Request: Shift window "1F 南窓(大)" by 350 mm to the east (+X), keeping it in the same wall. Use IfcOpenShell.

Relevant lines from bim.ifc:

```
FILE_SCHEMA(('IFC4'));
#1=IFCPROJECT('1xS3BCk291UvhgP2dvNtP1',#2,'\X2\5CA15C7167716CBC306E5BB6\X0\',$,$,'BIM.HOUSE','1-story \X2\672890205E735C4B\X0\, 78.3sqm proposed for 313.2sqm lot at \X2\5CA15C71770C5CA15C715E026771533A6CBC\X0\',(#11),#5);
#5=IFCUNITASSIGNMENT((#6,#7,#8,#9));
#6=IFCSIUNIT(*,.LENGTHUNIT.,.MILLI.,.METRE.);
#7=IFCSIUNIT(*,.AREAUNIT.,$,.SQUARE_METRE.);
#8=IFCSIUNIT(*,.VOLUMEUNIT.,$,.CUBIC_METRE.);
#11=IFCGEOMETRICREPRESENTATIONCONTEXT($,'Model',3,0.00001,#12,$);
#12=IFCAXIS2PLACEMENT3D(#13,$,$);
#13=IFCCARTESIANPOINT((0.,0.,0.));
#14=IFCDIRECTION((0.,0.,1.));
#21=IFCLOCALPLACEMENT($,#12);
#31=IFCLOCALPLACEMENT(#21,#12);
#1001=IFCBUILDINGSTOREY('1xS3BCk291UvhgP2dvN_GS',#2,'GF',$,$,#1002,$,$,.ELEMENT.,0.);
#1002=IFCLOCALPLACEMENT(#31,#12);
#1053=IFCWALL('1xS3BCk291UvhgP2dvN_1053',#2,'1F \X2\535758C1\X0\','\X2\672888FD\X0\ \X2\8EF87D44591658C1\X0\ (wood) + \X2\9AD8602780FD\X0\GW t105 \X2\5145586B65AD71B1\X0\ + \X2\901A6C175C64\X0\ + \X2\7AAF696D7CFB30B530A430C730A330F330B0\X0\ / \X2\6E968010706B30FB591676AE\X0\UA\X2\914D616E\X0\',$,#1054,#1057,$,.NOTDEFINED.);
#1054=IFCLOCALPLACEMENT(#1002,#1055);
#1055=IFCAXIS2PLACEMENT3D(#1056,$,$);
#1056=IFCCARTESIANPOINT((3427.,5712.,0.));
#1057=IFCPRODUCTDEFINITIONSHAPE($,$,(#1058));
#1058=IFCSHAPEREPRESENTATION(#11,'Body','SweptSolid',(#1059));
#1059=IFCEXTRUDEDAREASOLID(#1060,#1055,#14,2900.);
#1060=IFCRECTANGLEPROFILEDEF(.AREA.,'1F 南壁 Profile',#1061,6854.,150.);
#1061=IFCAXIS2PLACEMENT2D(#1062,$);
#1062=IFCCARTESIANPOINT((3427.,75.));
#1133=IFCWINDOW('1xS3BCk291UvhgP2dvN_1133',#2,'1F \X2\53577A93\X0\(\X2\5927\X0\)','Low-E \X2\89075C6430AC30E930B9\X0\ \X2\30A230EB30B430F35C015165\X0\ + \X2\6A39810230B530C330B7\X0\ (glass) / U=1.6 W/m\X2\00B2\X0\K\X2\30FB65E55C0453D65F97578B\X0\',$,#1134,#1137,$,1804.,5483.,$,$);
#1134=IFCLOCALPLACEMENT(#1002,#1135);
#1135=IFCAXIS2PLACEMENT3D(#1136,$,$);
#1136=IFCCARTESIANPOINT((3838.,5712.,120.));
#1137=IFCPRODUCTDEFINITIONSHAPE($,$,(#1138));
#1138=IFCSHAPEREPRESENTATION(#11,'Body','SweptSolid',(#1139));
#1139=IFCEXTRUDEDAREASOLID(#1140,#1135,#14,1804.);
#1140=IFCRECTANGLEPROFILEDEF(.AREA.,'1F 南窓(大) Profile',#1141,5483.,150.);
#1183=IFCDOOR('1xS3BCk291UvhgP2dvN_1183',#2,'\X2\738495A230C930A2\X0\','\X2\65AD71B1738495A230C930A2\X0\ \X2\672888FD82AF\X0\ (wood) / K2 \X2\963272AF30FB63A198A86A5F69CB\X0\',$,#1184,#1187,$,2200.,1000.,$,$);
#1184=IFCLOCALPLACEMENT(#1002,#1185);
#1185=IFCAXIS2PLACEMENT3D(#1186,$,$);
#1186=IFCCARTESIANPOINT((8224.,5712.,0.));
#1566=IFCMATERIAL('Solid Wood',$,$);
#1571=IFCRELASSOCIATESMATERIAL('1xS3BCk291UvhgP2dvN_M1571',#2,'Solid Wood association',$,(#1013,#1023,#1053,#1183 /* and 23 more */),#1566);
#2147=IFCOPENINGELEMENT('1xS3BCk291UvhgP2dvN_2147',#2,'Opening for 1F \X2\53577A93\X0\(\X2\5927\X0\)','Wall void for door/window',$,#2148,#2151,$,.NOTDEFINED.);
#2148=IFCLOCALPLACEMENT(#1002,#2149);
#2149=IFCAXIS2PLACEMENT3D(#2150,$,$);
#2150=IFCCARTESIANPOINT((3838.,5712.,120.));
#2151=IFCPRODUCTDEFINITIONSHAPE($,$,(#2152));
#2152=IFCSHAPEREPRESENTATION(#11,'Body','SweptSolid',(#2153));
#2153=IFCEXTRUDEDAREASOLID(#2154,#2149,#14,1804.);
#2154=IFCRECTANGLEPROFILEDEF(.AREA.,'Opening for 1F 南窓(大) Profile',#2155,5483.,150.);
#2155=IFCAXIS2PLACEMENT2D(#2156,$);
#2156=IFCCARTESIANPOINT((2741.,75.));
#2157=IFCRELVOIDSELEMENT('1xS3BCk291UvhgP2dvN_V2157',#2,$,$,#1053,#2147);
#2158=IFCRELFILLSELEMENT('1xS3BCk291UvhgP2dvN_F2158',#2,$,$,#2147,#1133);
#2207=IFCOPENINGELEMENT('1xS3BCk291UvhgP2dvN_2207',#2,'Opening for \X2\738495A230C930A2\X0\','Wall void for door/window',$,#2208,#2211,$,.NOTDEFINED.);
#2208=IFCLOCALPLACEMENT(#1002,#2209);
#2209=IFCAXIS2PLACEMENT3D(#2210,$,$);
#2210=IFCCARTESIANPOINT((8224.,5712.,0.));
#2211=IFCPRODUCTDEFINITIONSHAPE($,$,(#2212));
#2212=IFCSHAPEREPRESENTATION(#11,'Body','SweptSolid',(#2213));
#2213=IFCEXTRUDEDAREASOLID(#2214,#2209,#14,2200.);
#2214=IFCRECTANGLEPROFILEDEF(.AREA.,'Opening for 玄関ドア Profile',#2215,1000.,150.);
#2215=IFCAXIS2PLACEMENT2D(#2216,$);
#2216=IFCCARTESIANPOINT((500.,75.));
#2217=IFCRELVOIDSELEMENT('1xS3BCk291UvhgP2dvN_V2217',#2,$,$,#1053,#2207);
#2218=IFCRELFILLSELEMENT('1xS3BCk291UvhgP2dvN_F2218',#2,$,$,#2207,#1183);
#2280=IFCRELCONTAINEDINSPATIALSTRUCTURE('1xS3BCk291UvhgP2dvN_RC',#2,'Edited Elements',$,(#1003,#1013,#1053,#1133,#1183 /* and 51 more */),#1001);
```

```python
import ifcopenshell
import ifcopenshell.api.geometry
import ifcopenshell.util.placement
import ifcopenshell.util.unit

model = ifcopenshell.open("bim.ifc")
unit_scale = ifcopenshell.util.unit.calculate_unit_scale(model)

window = model.by_guid("1xS3BCk291UvhgP2dvN_1133")
opening = window.FillsVoids[0].RelatingOpeningElement
wall = opening.VoidsElements[0].RelatingBuildingElement

wall_matrix = ifcopenshell.util.placement.get_local_placement(wall.ObjectPlacement)
shift = wall_matrix[:3, 0] * 0.35 / unit_scale
before = ifcopenshell.util.placement.get_local_placement(window.ObjectPlacement)[:3, 3].copy()

# The window is not placed relative to its opening, so move both.
for product in (opening, window):
    matrix = ifcopenshell.util.placement.get_local_placement(product.ObjectPlacement)
    matrix[:3, 3] += shift
    ifcopenshell.api.geometry.edit_object_placement(model, product=product, matrix=matrix, is_si=False)

after = ifcopenshell.util.placement.get_local_placement(window.ObjectPlacement)[:3, 3]
print("window moved by", (after - before).round(3) + 0.0)

model.write("bim_v2.ifc")
```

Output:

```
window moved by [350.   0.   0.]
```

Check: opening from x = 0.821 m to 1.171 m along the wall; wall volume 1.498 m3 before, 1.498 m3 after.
